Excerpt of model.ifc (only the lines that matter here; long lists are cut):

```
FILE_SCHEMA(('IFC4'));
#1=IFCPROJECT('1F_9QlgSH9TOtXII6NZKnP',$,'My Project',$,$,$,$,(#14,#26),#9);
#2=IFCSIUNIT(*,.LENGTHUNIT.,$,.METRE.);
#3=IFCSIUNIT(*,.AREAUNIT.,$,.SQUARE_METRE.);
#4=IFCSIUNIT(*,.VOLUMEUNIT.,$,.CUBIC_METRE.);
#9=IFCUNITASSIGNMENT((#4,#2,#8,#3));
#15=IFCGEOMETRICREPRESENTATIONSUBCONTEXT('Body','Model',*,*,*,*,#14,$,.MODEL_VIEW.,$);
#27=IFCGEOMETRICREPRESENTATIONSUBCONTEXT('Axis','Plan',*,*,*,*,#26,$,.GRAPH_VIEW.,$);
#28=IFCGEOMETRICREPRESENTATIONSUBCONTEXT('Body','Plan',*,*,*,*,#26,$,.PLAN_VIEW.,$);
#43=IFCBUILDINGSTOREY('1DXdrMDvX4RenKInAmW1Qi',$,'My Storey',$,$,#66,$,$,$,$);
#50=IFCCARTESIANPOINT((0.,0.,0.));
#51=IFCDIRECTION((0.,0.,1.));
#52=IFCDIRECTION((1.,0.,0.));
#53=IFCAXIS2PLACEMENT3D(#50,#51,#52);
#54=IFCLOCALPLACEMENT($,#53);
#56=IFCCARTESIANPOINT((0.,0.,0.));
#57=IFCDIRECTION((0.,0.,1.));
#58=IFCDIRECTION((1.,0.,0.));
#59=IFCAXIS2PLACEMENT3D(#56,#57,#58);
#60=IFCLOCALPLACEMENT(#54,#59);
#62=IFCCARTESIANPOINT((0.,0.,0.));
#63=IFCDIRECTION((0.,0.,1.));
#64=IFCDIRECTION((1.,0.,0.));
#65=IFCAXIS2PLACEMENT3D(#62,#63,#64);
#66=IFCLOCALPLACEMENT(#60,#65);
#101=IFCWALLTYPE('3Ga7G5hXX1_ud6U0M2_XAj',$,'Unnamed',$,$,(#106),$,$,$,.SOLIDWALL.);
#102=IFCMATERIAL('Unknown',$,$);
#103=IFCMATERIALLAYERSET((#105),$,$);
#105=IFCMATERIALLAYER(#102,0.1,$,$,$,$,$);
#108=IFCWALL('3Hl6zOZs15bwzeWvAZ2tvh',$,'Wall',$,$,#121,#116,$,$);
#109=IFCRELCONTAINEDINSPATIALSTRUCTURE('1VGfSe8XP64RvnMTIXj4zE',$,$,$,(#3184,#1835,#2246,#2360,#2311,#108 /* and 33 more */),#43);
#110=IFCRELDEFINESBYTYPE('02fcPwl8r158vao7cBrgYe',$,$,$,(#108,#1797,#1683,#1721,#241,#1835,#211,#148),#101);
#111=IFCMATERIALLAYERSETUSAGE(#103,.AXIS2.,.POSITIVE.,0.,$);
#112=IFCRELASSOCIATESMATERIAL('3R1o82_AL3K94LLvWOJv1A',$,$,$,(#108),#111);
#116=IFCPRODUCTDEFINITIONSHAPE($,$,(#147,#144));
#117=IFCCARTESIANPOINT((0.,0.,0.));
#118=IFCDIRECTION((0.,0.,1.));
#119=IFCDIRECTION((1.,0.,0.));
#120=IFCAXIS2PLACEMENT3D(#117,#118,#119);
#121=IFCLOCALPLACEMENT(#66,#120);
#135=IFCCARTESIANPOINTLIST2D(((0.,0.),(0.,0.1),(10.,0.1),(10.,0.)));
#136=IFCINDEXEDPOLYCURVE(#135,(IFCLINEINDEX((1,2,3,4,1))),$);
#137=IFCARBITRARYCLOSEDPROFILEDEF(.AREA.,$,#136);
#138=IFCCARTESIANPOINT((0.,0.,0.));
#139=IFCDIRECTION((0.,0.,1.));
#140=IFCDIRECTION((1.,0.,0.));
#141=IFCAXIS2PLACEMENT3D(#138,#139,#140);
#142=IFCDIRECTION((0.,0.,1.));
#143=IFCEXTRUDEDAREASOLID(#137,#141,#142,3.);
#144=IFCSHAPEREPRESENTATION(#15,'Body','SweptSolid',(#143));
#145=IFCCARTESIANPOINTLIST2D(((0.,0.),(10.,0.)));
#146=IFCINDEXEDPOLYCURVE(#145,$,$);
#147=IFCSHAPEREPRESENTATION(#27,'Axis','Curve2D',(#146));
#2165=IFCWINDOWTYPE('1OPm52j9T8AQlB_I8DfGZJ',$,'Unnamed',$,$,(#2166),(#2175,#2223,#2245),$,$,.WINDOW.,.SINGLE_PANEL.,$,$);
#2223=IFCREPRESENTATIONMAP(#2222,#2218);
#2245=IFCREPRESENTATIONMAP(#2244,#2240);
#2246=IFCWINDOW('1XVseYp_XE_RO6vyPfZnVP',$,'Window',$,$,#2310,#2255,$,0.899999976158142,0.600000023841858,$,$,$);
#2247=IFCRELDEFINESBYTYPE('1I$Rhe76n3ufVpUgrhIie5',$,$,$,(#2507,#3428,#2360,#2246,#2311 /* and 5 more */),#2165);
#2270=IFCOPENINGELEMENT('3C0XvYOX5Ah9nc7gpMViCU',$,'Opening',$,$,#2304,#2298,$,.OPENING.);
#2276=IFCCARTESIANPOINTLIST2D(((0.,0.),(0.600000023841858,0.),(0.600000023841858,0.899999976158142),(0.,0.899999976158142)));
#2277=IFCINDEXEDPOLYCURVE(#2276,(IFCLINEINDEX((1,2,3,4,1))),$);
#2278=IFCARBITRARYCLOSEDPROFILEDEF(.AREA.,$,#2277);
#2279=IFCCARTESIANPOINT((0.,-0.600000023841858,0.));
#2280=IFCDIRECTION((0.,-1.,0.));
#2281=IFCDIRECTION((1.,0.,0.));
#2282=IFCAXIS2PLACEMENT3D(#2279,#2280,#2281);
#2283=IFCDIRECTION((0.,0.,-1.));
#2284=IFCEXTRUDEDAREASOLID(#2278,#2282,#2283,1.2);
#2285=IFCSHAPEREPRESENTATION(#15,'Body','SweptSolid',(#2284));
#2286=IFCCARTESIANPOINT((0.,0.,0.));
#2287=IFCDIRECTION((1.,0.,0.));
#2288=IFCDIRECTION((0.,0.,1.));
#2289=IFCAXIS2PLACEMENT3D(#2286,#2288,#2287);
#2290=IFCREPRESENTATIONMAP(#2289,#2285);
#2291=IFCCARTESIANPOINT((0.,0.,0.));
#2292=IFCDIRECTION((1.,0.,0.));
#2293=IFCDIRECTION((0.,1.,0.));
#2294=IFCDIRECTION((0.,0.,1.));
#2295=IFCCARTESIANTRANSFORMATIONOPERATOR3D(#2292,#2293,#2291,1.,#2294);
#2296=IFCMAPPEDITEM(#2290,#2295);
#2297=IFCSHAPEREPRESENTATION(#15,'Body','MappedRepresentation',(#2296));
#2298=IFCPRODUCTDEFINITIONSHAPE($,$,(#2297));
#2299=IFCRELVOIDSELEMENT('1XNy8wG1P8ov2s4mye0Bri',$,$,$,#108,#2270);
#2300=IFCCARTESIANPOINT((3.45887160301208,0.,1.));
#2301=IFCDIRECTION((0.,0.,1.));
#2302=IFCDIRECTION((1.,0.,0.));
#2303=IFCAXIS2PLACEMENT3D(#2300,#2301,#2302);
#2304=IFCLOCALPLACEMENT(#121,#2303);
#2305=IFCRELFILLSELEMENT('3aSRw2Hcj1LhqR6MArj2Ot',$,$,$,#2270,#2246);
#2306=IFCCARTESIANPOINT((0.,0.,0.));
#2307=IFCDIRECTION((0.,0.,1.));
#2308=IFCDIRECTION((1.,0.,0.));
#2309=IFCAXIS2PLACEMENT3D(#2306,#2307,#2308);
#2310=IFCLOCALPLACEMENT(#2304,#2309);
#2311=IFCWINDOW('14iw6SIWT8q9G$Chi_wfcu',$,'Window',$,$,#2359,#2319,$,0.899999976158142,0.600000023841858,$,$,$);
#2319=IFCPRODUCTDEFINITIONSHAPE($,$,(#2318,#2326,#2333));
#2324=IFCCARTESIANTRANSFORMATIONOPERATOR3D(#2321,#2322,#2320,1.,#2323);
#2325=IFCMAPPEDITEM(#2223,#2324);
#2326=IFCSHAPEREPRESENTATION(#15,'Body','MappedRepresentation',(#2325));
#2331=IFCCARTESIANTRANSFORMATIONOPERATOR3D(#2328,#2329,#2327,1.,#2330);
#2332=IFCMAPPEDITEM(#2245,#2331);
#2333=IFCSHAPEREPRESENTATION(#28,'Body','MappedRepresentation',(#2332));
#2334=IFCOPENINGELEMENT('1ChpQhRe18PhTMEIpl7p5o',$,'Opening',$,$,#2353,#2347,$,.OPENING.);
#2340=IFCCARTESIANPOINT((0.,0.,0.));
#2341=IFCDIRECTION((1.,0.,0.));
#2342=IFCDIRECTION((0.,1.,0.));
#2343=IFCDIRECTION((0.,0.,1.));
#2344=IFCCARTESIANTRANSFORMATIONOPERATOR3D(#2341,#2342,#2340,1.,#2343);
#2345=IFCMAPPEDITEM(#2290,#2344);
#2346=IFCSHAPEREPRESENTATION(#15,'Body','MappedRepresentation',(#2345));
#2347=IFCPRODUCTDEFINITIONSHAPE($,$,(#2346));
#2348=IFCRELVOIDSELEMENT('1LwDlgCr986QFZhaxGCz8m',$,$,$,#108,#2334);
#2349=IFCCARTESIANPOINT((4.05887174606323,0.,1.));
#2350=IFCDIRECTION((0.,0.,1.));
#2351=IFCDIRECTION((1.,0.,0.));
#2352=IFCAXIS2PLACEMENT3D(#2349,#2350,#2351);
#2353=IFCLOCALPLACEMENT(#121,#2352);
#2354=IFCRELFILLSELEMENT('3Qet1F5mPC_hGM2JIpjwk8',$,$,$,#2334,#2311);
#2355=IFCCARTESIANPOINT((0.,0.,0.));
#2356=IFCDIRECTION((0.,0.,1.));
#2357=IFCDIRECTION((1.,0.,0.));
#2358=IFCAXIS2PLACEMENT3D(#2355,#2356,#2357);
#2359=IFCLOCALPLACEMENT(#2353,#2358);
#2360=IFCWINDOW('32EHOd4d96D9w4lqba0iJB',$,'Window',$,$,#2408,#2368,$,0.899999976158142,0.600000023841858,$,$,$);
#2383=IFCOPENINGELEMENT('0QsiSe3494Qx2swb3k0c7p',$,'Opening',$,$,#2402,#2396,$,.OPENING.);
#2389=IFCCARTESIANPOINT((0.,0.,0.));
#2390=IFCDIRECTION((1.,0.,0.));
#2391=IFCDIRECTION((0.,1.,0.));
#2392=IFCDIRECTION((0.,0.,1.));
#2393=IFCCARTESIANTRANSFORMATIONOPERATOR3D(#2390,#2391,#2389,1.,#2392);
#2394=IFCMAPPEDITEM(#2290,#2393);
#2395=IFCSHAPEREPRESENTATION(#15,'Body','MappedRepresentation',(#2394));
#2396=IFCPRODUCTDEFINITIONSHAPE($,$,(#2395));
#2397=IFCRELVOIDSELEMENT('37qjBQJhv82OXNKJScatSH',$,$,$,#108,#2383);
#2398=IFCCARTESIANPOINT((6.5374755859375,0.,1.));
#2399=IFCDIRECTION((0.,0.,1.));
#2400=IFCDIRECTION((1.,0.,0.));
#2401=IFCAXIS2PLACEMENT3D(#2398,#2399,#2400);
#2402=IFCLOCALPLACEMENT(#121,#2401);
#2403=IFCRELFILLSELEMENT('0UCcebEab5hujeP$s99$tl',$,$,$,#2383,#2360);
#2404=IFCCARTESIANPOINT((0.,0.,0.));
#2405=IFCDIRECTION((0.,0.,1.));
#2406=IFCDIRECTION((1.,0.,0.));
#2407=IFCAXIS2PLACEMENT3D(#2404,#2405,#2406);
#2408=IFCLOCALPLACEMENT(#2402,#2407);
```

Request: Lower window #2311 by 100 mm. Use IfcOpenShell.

```python
import numpy as np
import ifcopenshell
import ifcopenshell.api.geometry
import ifcopenshell.util.placement
import ifcopenshell.util.unit

model = ifcopenshell.open("model.ifc")
unit_scale = ifcopenshell.util.unit.calculate_unit_scale(model)

window = model.by_guid("14iw6SIWT8q9G$Chi_wfcu")
opening = window.FillsVoids[0].RelatingOpeningElement
dz = -0.1

shift = np.array([0.0, 0.0, dz])
# The window is placed relative to its opening, so it follows when the opening moves.
matrix = ifcopenshell.util.placement.get_local_placement(opening.ObjectPlacement)
matrix[:3, 3] += shift
ifcopenshell.api.geometry.edit_object_placement(
    model, product=opening, matrix=matrix, is_si=False, should_transform_children=True
)

print(f"moved by {dz * unit_scale:+.3f} m")

model.write("model_updated.ifc")
```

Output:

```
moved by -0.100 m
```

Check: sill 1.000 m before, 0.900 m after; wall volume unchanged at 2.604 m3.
